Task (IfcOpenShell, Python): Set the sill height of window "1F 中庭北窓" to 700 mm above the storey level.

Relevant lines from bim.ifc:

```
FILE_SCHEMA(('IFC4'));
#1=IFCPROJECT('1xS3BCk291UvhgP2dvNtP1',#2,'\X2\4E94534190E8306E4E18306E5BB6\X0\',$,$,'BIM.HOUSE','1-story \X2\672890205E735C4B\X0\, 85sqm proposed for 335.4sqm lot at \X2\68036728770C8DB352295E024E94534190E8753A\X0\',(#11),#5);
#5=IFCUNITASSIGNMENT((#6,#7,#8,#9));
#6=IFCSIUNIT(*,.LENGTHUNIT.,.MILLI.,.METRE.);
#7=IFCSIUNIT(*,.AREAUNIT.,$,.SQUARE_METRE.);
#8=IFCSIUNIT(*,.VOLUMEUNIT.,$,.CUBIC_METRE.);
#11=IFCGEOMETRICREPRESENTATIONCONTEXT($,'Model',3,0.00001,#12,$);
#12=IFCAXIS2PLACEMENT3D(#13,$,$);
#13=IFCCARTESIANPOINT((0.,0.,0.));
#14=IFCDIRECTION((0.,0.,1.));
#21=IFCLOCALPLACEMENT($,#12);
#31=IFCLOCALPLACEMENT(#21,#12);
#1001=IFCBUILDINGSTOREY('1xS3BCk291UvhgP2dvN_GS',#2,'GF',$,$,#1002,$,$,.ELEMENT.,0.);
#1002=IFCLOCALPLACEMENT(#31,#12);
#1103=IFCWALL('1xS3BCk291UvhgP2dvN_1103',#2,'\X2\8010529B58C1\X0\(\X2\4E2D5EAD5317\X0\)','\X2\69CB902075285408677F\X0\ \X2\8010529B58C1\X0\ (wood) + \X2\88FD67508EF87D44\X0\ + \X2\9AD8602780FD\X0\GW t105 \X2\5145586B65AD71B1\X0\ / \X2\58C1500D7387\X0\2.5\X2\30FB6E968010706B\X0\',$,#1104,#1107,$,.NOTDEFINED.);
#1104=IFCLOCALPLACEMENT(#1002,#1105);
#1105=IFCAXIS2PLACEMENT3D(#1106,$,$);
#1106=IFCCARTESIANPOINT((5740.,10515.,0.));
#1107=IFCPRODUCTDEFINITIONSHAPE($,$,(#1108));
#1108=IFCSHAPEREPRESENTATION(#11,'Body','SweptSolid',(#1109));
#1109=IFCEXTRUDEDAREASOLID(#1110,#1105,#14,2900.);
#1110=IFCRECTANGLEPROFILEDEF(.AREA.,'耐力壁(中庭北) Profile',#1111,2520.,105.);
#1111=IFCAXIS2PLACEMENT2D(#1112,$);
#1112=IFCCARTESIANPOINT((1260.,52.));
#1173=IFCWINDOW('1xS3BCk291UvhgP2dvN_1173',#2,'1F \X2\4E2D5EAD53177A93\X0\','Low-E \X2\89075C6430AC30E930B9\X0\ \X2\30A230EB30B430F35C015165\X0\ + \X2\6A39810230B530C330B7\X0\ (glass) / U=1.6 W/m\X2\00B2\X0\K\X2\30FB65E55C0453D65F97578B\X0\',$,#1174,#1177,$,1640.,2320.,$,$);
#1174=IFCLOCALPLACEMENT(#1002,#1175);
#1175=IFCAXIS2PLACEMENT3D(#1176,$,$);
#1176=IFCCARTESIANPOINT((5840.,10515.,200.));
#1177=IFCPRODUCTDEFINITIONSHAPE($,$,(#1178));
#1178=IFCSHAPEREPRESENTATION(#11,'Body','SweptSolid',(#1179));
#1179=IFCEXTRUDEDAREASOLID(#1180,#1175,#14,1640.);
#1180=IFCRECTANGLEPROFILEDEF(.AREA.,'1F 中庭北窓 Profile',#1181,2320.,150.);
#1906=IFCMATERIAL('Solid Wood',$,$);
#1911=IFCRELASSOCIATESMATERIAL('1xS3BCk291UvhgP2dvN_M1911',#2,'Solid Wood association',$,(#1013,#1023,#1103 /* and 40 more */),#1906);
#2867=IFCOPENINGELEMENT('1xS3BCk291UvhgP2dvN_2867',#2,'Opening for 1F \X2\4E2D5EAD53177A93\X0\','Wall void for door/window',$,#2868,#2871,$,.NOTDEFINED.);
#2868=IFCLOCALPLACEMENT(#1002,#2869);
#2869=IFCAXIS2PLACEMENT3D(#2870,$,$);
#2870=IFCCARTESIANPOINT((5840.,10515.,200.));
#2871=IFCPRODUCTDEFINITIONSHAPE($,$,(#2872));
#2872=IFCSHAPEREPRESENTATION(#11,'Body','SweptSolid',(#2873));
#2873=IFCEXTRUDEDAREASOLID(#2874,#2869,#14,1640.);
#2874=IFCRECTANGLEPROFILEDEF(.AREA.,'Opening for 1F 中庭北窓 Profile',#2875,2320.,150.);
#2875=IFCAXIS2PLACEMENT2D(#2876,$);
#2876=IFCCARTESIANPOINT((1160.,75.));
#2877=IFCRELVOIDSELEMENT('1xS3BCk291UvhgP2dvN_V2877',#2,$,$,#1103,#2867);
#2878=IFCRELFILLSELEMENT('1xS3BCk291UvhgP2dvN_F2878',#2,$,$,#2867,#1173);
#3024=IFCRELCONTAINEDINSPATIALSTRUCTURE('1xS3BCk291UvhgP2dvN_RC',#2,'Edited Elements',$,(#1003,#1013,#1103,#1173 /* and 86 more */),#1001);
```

```python
import numpy as np
import ifcopenshell
import ifcopenshell.api.geometry
import ifcopenshell.geom
import ifcopenshell.util.element
import ifcopenshell.util.placement
import ifcopenshell.util.shape
import ifcopenshell.util.unit

model = ifcopenshell.open("bim.ifc")
unit_scale = ifcopenshell.util.unit.calculate_unit_scale(model)

window = model.by_guid("1xS3BCk291UvhgP2dvN_1173")
opening = window.FillsVoids[0].RelatingOpeningElement
storey = ifcopenshell.util.element.get_container(window, ifc_class="IfcBuildingStorey")
level = ifcopenshell.util.placement.get_local_placement(storey.ObjectPlacement)[2, 3]

# The opening's origin need not be at the sill, so measure its lowest point.
shape = ifcopenshell.geom.create_shape(ifcopenshell.geom.settings(), opening)
bottom = ifcopenshell.util.shape.get_shape_bottom_elevation(shape, shape.geometry) / unit_scale
dz = level + 700.0 - bottom

shift = np.array([0.0, 0.0, dz])
# The window is not placed relative to its opening, so move both.
for product in (opening, window):
    matrix = ifcopenshell.util.placement.get_local_placement(product.ObjectPlacement)
    matrix[:3, 3] += shift
    ifcopenshell.api.geometry.edit_object_placement(model, product=product, matrix=matrix, is_si=False)

print(f"moved by {dz * unit_scale:+.3f} m")

model.write("bim_updated.ifc")
```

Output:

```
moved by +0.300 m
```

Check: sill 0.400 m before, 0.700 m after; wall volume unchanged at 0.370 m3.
